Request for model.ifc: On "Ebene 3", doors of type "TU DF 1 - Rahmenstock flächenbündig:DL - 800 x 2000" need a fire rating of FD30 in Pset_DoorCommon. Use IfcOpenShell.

First a look at what the model holds.

```python
import ifcopenshell
import ifcopenshell.util.element

model = ifcopenshell.open("model.ifc")
print(model.schema)
storey = next(s for s in model.by_type("IfcBuildingStorey") if s.Name == "Ebene 3")
doors = [e for e in ifcopenshell.util.element.get_decomposition(storey) if e.is_a("IfcDoor")]
seen = {}
for e in doors:
    element_type = ifcopenshell.util.element.get_type(e)
    key = (element_type.Name if element_type != e and element_type else None, ifcopenshell.util.element.get_pset(e, "Pset_DoorCommon", "FireRating"))
    seen[key] = seen.get(key, 0) + 1
for (name, value), count in sorted(seen.items(), key=str):
    print(count, "x", name, "|", value)
```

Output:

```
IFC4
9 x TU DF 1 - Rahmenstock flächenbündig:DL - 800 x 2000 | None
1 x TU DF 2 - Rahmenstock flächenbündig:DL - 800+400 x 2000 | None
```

```python
import ifcopenshell
import ifcopenshell.api.pset
import ifcopenshell.util.element

model = ifcopenshell.open("model.ifc")

storey = next(s for s in model.by_type("IfcBuildingStorey") if s.Name == "Ebene 3")
doors = [e for e in ifcopenshell.util.element.get_decomposition(storey) if e.is_a("IfcDoor")]

count = 0
for e in doors:
    element_type = ifcopenshell.util.element.get_type(e)
    if element_type in (None, e) or element_type.Name != "TU DF 1 - Rahmenstock flächenbündig:DL - 800 x 2000":
        continue
    # add_pset returns the element's existing set when there is one.
    pset = ifcopenshell.api.pset.add_pset(model, product=e, name="Pset_DoorCommon")
    ifcopenshell.api.pset.edit_pset(model, pset=pset, properties={"FireRating": "FD30"})
    count += 1

print(count, "doors updated")

model.write("model_edited.ifc")
```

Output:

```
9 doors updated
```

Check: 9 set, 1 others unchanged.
